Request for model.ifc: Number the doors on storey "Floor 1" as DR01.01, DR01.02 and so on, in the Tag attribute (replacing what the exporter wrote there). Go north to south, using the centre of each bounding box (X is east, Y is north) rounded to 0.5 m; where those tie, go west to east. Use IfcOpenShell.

First a look at what the model holds.

```python
import ifcopenshell
import ifcopenshell.util.element
import ifcopenshell.util.placement

model = ifcopenshell.open("model.ifc")
print(model.schema)
storey = next(s for s in model.by_type("IfcBuildingStorey") if s.Name == "Floor 1")
doors = [e for e in ifcopenshell.util.element.get_decomposition(storey) if e.is_a("IfcDoor")]
for e in sorted(doors, key=lambda e: e.id()):
    origin = ifcopenshell.util.placement.get_local_placement(e.ObjectPlacement)[:3, 3]
    print(e.id(), e.Tag, e.Name, origin.round(2) + 0.0, sep=" | ")
```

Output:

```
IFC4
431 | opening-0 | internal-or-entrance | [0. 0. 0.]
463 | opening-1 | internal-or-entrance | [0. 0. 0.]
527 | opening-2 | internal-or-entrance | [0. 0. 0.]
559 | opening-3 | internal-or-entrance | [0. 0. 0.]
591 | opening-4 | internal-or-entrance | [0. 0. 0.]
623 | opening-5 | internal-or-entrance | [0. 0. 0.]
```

```python
import ifcopenshell
import ifcopenshell.geom
import ifcopenshell.util.element
import ifcopenshell.util.shape

model = ifcopenshell.open("model.ifc")
settings = ifcopenshell.geom.settings()
settings.set("use-world-coords", True)


def centre(element):
    shape = ifcopenshell.geom.create_shape(settings, element)
    return ifcopenshell.util.shape.get_bbox_centroid(shape.geometry)


storey = next(s for s in model.by_type("IfcBuildingStorey") if s.Name == "Floor 1")
doors = [e for e in ifcopenshell.util.element.get_decomposition(storey) if e.is_a("IfcDoor")]

# Insertion points can sit at a corner or the storey origin, so sort by the geometry (in metres).
centres = {e: centre(e) for e in doors}
doors.sort(key=lambda e: (-round(centres[e][1] / 0.5), centres[e][0]))

for i, e in enumerate(doors, start=1):
    number = f"DR01.{i:02d}"
    e.Tag = number
    print(e.id(), number)

model.write("model_edited.ifc")
```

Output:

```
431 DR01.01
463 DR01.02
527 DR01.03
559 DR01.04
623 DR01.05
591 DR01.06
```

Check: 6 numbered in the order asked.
